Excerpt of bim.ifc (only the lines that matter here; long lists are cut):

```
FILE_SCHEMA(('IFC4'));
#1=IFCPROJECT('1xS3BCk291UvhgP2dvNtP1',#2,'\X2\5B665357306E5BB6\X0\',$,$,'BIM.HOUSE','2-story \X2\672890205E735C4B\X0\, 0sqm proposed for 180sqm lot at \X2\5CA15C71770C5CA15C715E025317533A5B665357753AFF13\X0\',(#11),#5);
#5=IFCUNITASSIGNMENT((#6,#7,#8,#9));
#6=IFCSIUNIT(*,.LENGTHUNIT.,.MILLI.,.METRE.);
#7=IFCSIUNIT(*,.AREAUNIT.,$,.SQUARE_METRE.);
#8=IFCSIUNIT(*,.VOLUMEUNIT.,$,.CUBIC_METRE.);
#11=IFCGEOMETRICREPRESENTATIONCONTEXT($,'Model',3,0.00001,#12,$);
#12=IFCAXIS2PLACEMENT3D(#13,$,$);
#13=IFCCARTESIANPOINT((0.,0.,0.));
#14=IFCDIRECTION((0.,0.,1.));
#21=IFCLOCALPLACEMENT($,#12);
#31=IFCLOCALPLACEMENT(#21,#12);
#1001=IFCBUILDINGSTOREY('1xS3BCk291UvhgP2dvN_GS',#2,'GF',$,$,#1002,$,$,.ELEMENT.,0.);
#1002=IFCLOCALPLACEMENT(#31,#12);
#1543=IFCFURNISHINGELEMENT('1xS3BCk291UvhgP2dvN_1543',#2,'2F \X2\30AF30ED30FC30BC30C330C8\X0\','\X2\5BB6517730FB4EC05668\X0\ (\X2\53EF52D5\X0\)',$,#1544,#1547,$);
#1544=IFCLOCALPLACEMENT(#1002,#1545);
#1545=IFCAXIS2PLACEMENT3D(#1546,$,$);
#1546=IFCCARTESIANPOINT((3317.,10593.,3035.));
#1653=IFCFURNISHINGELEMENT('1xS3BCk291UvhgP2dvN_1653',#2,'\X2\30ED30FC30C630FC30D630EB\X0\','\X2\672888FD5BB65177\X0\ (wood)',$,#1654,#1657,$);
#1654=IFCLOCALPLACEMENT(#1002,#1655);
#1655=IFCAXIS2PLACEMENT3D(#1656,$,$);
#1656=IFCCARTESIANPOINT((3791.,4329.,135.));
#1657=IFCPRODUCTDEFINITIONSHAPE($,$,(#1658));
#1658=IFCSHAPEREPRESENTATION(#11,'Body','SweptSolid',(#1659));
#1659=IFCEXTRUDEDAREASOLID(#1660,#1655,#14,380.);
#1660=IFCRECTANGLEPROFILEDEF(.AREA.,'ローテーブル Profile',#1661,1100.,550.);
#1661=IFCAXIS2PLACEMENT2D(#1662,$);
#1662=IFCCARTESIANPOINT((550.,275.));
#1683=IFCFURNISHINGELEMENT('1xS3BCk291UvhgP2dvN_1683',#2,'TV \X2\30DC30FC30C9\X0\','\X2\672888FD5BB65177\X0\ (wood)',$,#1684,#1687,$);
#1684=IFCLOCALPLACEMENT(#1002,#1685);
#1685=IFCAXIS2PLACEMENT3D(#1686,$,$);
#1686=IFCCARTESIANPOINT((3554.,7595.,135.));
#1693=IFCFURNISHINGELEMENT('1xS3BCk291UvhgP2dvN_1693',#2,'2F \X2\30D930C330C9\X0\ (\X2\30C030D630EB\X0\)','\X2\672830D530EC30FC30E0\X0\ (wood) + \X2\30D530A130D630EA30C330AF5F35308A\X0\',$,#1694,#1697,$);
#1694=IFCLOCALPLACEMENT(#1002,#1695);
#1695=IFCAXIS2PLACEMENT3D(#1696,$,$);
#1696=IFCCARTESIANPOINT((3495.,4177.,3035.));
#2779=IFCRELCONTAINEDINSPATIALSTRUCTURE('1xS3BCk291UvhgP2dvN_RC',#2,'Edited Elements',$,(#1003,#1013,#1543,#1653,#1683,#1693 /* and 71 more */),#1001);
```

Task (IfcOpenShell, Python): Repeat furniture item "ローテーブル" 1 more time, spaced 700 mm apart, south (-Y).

```python
import numpy as np
import ifcopenshell
import ifcopenshell.api.geometry
import ifcopenshell.api.root
import ifcopenshell.util.element
import ifcopenshell.util.placement
import ifcopenshell.util.unit

model = ifcopenshell.open("bim.ifc")
unit_scale = ifcopenshell.util.unit.calculate_unit_scale(model)


def reuse_history(source, copy):
    """copy_class also copies each property set's owner history, people and application; keep the originals."""
    for rel in copy.IsDefinedBy:
        if rel.is_a("IfcRelDefinesByProperties") and (history := rel.RelatingPropertyDefinition.OwnerHistory):
            rel.RelatingPropertyDefinition.OwnerHistory = source.OwnerHistory
            ifcopenshell.util.element.remove_deep2(model, history)


source = model.by_id(1653)
base = ifcopenshell.util.placement.get_local_placement(source.ObjectPlacement)
step = np.array([0.0, -1.0, 0.0]) * 0.7 / unit_scale

for i in range(1, 2):
    copy = ifcopenshell.api.root.copy_class(model, product=source)
    copy.Representation = ifcopenshell.util.element.copy_deep(
        model, source.Representation, exclude=["IfcGeometricRepresentationContext", "IfcRepresentationMap"]
    )
    reuse_history(source, copy)
    matrix = base.copy()
    matrix[:3, 3] += i * step
    print("added at", matrix[:3, 3].round(3) + 0.0)
    ifcopenshell.api.geometry.edit_object_placement(model, product=copy, matrix=matrix, is_si=False)

model.write("bim-out.ifc")
```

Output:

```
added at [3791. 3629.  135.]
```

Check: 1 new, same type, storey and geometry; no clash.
